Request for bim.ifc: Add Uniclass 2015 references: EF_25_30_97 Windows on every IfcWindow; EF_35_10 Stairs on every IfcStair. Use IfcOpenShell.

First a look at what the model holds.

```python
import ifcopenshell

model = ifcopenshell.open("bim.ifc")
print(model.schema)
print("classifications:", [c.Name for c in model.by_type("IfcClassification")])
for ifc_class in ("IfcDoor", "IfcRoof", "IfcStair", "IfcWall", "IfcWindow"):
    print(ifc_class, len(model.by_type(ifc_class)))
```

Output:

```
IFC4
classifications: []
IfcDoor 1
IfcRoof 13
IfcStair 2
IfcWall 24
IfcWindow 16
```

```python
import ifcopenshell
import ifcopenshell.api.classification

model = ifcopenshell.open("bim.ifc")

system = ifcopenshell.api.classification.add_classification(model, classification="Uniclass 2015")

codes = {
    "IfcWindow": ("EF_25_30_97", "Windows"),
    "IfcStair": ("EF_35_10", "Stairs"),
}
for ifc_class, (code, name) in codes.items():
    products = model.by_type(ifc_class)
    ifcopenshell.api.classification.add_reference(
        model, products=products, classification=system, identification=code, name=name
    )
    print(code, len(products))

model.write("bim_edited.ifc")
```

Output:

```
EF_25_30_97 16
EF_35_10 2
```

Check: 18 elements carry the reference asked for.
